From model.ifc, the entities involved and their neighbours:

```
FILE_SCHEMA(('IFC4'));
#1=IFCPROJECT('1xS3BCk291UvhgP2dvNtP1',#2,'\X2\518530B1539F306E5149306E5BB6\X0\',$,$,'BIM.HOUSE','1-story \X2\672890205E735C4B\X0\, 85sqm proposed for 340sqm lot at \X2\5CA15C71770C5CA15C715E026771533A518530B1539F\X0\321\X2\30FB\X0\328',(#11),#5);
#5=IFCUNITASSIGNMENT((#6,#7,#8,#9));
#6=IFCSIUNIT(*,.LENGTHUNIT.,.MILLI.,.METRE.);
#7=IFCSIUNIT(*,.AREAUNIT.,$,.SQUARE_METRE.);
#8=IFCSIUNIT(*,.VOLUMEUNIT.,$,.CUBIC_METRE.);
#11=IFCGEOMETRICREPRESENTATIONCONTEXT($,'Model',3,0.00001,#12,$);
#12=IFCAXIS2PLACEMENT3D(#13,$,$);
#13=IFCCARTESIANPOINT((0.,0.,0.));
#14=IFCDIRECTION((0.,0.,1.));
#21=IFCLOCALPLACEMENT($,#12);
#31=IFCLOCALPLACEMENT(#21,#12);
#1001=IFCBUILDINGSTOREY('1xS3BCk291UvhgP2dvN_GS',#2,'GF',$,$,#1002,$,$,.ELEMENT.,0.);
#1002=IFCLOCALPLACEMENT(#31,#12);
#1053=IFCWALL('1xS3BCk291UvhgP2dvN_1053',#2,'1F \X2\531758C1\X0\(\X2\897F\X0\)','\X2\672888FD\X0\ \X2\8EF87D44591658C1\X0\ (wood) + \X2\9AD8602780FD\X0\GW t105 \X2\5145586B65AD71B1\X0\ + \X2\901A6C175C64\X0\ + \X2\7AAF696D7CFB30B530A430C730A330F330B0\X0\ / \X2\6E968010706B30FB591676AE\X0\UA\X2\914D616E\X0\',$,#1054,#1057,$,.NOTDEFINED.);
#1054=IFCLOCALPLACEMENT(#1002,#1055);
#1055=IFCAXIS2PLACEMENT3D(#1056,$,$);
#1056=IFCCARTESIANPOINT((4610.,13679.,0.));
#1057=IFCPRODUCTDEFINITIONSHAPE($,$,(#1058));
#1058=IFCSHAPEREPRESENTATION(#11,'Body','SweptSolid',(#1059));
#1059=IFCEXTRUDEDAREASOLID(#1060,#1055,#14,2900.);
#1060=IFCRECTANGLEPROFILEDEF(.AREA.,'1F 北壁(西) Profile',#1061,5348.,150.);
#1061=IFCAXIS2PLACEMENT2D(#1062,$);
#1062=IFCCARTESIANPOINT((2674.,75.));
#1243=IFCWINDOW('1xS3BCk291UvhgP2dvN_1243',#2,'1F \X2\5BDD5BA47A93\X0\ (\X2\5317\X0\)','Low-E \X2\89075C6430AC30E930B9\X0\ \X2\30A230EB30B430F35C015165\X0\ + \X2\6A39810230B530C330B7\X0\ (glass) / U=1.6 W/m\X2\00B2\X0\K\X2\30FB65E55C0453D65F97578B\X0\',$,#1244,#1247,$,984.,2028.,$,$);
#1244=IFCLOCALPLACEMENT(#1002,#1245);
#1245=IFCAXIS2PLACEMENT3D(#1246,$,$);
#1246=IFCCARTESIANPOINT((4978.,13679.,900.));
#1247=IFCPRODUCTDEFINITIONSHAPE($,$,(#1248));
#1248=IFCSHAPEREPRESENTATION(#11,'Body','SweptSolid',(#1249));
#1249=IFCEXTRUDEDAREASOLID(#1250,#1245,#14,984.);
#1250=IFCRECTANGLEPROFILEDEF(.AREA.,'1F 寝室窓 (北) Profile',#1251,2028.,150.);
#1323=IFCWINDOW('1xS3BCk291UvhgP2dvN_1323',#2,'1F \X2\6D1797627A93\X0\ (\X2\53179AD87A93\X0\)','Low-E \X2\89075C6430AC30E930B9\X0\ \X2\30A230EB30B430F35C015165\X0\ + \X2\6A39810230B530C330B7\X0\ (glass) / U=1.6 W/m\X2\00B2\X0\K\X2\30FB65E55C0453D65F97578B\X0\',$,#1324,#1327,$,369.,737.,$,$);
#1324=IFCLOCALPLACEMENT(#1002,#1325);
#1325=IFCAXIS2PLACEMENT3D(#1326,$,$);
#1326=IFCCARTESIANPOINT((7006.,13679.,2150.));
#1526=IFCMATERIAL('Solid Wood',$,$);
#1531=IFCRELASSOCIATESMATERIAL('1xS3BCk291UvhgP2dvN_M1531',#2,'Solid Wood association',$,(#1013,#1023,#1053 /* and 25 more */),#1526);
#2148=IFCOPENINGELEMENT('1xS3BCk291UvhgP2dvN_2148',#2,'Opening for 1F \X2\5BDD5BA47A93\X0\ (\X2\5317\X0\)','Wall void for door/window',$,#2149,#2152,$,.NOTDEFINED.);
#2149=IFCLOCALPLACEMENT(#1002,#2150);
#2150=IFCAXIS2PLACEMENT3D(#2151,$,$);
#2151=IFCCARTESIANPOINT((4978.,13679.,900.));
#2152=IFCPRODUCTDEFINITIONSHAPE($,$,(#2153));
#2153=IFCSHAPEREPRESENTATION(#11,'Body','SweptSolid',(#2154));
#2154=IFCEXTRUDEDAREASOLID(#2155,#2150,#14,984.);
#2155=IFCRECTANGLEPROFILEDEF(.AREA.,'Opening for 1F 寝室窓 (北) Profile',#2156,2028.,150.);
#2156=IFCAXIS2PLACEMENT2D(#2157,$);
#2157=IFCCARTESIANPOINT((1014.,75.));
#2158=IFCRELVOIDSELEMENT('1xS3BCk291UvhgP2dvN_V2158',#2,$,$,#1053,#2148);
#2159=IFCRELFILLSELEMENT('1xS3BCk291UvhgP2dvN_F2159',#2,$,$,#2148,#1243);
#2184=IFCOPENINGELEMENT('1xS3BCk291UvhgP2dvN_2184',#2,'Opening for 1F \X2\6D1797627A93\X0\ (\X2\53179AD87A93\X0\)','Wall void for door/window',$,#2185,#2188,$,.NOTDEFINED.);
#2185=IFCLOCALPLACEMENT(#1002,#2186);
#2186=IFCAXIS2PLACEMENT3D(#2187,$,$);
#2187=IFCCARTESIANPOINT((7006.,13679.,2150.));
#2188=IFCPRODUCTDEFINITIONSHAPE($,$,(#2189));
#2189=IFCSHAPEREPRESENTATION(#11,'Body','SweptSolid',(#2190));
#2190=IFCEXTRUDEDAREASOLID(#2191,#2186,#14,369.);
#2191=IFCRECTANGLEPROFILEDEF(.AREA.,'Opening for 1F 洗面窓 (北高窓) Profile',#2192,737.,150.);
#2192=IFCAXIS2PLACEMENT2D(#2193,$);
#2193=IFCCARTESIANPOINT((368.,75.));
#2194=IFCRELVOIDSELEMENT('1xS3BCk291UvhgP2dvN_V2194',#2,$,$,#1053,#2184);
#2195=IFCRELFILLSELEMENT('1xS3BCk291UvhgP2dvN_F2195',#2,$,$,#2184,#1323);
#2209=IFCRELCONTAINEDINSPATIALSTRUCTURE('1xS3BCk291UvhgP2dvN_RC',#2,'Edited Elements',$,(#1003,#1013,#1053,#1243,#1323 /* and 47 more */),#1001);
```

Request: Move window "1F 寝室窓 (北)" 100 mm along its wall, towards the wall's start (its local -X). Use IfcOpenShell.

```python
import ifcopenshell
import ifcopenshell.api.geometry
import ifcopenshell.util.placement
import ifcopenshell.util.unit

model = ifcopenshell.open("model.ifc")
unit_scale = ifcopenshell.util.unit.calculate_unit_scale(model)

window = model.by_guid("1xS3BCk291UvhgP2dvN_1243")
opening = window.FillsVoids[0].RelatingOpeningElement
wall = opening.VoidsElements[0].RelatingBuildingElement

wall_matrix = ifcopenshell.util.placement.get_local_placement(wall.ObjectPlacement)
shift = wall_matrix[:3, 0] * -0.1 / unit_scale
before = ifcopenshell.util.placement.get_local_placement(window.ObjectPlacement)[:3, 3].copy()

# The window is not placed relative to its opening, so move both.
for product in (opening, window):
    matrix = ifcopenshell.util.placement.get_local_placement(product.ObjectPlacement)
    matrix[:3, 3] += shift
    ifcopenshell.api.geometry.edit_object_placement(model, product=product, matrix=matrix, is_si=False)

after = ifcopenshell.util.placement.get_local_placement(window.ObjectPlacement)[:3, 3]
print("window moved by", (after - before).round(3) + 0.0)

model.write("model-out.ifc")
```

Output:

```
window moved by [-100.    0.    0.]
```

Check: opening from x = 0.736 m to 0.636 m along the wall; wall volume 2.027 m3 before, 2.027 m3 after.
